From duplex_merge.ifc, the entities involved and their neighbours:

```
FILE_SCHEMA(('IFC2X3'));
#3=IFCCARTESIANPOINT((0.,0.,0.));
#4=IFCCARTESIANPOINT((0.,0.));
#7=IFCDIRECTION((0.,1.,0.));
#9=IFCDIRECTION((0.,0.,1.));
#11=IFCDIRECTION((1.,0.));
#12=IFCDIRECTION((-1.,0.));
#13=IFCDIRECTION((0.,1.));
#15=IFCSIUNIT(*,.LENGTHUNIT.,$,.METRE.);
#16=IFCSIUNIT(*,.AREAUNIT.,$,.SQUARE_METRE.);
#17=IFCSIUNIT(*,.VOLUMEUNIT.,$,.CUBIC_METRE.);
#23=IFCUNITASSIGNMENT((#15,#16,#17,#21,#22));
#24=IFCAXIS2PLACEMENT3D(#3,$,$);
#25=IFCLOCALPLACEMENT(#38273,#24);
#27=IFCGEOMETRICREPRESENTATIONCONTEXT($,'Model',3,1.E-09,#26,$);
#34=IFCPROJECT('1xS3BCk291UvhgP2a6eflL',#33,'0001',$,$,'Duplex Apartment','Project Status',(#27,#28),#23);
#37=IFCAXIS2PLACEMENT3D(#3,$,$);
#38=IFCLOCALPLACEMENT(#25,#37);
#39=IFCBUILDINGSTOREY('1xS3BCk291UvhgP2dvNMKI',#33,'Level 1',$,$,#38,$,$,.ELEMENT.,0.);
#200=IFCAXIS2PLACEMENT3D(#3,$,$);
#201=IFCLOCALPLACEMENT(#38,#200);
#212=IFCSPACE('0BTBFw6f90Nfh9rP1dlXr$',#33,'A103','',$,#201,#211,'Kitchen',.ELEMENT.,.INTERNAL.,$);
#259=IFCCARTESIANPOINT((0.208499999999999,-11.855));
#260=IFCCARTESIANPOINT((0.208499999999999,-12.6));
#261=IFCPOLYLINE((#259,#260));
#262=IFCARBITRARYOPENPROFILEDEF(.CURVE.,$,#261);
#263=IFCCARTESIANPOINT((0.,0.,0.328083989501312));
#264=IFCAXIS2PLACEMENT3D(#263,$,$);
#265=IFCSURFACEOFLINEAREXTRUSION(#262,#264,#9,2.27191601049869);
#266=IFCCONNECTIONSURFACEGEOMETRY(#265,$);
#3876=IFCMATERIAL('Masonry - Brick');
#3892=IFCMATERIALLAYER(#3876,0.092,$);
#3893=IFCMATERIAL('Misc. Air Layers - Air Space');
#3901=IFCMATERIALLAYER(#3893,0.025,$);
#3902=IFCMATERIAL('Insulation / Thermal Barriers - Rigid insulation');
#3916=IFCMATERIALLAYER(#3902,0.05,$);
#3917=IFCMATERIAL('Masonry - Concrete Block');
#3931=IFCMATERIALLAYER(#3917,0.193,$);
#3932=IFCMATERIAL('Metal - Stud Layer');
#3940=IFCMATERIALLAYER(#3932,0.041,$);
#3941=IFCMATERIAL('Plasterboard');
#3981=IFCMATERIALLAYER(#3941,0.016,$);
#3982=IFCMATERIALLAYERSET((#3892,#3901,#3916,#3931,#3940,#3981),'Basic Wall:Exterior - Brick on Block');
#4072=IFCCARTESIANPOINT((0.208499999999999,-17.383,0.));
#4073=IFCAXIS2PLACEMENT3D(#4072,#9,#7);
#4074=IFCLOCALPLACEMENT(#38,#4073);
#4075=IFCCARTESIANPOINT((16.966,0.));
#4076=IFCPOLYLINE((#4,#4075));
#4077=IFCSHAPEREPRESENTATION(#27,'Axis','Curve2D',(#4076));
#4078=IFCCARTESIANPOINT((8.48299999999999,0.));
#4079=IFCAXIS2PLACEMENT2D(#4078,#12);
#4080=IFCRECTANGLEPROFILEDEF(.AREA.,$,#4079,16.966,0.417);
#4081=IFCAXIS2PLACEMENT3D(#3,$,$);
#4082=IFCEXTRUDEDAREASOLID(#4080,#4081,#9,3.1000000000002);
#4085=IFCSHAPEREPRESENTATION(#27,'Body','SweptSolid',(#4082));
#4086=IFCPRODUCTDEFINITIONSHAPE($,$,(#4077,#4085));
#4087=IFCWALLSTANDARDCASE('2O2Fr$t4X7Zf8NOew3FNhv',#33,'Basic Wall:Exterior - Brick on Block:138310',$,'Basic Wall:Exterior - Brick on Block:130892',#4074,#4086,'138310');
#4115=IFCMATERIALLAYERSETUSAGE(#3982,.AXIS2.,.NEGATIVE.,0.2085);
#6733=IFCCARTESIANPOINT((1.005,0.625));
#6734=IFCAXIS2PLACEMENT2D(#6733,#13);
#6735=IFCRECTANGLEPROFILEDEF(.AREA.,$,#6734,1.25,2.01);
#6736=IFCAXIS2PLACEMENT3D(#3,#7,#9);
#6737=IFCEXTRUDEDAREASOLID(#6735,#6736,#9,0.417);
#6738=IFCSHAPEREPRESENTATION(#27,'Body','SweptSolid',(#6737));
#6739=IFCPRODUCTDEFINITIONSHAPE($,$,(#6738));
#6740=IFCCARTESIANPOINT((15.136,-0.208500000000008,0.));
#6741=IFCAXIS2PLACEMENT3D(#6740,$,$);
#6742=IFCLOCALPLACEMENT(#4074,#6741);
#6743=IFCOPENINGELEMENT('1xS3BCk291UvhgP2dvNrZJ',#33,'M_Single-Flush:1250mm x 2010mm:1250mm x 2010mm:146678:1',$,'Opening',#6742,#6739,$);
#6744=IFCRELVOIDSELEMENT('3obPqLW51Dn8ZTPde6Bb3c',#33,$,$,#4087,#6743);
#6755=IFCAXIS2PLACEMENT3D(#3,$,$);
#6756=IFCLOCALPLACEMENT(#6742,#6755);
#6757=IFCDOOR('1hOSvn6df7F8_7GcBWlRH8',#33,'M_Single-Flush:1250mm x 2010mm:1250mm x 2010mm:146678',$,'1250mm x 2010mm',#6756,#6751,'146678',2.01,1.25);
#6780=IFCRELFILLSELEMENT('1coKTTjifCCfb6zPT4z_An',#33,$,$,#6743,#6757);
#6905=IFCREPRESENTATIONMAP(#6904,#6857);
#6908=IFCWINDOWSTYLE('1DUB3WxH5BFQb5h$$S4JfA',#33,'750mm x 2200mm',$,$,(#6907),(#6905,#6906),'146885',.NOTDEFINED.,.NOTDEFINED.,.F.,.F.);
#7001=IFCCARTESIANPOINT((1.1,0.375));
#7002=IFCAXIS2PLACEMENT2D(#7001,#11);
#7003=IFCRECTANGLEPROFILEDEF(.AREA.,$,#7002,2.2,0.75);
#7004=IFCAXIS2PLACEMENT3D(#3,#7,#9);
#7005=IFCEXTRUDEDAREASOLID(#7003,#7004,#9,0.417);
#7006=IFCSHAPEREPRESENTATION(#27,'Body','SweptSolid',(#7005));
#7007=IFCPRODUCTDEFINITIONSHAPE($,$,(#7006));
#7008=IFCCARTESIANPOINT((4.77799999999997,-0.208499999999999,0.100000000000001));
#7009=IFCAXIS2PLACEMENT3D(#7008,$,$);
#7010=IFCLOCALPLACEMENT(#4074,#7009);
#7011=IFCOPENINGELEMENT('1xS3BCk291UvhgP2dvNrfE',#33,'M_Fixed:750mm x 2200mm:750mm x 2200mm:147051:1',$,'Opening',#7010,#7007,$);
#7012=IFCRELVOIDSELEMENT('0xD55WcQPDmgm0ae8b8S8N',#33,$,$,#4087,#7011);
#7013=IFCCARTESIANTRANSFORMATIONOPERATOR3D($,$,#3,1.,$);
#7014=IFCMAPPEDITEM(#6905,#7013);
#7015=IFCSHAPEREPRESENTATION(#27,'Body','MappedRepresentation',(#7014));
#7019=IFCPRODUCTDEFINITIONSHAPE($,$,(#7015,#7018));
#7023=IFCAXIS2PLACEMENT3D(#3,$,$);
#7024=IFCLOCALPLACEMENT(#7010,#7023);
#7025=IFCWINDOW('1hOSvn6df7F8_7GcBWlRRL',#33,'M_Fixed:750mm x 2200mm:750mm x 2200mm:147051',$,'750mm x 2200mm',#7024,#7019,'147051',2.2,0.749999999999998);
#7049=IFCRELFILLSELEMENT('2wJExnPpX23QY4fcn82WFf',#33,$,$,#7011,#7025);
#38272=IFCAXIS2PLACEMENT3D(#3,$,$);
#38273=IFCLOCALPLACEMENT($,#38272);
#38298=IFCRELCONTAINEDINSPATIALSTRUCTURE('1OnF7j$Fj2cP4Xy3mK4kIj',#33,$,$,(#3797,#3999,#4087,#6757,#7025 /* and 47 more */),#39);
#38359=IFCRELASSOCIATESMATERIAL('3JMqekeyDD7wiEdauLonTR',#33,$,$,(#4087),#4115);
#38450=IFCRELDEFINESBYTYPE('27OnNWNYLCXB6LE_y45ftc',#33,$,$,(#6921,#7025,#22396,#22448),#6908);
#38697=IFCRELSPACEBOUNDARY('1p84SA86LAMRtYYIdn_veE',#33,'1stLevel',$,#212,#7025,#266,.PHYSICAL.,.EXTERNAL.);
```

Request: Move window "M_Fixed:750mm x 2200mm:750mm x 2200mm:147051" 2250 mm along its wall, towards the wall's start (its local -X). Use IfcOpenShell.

```python
import numpy as np
import ifcopenshell
import ifcopenshell.api.geometry
import ifcopenshell.util.placement

model = ifcopenshell.open("duplex_merge.ifc")

window = model.by_id(7025)
opening = window.FillsVoids[0].RelatingOpeningElement
wall = opening.VoidsElements[0].RelatingBuildingElement

wall_matrix = ifcopenshell.util.placement.get_local_placement(wall.ObjectPlacement)
shift = wall_matrix[:3, 0] * -2.25
before = ifcopenshell.util.placement.get_local_placement(window.ObjectPlacement)[:3, 3].copy()

# The window is placed relative to its opening, so it follows when the opening moves.
matrix = ifcopenshell.util.placement.get_local_placement(opening.ObjectPlacement)
matrix[:3, 3] += shift
ifcopenshell.api.geometry.edit_object_placement(
    model, product=opening, matrix=matrix, is_si=False, should_transform_children=True
)

# Space boundary surfaces are stored in each space's coordinates; move them too.
for rel in window.ProvidesBoundaries:
    if not rel.ConnectionGeometry:
        continue
    surface = rel.ConnectionGeometry.SurfaceOnRelatingElement
    space_matrix = ifcopenshell.util.placement.get_local_placement(rel.RelatingSpace.ObjectPlacement)
    point = np.array(surface.Position.Location.Coordinates) + space_matrix[:3, :3].T @ shift
    surface.Position = model.createIfcAxis2Placement3D(
        model.createIfcCartesianPoint(point.tolist()), surface.Position.Axis, surface.Position.RefDirection
    )

after = ifcopenshell.util.placement.get_local_placement(window.ObjectPlacement)[:3, 3]
print("window moved by", (after - before).round(3) + 0.0)

model.write("duplex_merge-out.ifc")
```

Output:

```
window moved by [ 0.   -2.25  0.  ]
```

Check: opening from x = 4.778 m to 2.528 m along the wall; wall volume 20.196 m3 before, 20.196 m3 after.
